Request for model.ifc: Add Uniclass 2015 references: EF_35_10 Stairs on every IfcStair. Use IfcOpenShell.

First a look at what the model holds.

```python
import ifcopenshell

model = ifcopenshell.open("model.ifc")
print(model.schema)
print("classifications:", [c.Name for c in model.by_type("IfcClassification")])
for ifc_class in ("IfcDoor", "IfcRoof", "IfcStair", "IfcWall", "IfcWindow"):
    print(ifc_class, len(model.by_type(ifc_class)))
```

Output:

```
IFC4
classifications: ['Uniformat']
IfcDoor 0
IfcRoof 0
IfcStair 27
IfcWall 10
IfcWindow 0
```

```python
import ifcopenshell
import ifcopenshell.api.classification

model = ifcopenshell.open("model.ifc")

system = ifcopenshell.api.classification.add_classification(model, classification="Uniclass 2015")

codes = {
    "IfcStair": ("EF_35_10", "Stairs"),
}
for ifc_class, (code, name) in codes.items():
    products = model.by_type(ifc_class)
    ifcopenshell.api.classification.add_reference(
        model, products=products, classification=system, identification=code, name=name
    )
    print(code, len(products))

model.write("model_updated.ifc")
```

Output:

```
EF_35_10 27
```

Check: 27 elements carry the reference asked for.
